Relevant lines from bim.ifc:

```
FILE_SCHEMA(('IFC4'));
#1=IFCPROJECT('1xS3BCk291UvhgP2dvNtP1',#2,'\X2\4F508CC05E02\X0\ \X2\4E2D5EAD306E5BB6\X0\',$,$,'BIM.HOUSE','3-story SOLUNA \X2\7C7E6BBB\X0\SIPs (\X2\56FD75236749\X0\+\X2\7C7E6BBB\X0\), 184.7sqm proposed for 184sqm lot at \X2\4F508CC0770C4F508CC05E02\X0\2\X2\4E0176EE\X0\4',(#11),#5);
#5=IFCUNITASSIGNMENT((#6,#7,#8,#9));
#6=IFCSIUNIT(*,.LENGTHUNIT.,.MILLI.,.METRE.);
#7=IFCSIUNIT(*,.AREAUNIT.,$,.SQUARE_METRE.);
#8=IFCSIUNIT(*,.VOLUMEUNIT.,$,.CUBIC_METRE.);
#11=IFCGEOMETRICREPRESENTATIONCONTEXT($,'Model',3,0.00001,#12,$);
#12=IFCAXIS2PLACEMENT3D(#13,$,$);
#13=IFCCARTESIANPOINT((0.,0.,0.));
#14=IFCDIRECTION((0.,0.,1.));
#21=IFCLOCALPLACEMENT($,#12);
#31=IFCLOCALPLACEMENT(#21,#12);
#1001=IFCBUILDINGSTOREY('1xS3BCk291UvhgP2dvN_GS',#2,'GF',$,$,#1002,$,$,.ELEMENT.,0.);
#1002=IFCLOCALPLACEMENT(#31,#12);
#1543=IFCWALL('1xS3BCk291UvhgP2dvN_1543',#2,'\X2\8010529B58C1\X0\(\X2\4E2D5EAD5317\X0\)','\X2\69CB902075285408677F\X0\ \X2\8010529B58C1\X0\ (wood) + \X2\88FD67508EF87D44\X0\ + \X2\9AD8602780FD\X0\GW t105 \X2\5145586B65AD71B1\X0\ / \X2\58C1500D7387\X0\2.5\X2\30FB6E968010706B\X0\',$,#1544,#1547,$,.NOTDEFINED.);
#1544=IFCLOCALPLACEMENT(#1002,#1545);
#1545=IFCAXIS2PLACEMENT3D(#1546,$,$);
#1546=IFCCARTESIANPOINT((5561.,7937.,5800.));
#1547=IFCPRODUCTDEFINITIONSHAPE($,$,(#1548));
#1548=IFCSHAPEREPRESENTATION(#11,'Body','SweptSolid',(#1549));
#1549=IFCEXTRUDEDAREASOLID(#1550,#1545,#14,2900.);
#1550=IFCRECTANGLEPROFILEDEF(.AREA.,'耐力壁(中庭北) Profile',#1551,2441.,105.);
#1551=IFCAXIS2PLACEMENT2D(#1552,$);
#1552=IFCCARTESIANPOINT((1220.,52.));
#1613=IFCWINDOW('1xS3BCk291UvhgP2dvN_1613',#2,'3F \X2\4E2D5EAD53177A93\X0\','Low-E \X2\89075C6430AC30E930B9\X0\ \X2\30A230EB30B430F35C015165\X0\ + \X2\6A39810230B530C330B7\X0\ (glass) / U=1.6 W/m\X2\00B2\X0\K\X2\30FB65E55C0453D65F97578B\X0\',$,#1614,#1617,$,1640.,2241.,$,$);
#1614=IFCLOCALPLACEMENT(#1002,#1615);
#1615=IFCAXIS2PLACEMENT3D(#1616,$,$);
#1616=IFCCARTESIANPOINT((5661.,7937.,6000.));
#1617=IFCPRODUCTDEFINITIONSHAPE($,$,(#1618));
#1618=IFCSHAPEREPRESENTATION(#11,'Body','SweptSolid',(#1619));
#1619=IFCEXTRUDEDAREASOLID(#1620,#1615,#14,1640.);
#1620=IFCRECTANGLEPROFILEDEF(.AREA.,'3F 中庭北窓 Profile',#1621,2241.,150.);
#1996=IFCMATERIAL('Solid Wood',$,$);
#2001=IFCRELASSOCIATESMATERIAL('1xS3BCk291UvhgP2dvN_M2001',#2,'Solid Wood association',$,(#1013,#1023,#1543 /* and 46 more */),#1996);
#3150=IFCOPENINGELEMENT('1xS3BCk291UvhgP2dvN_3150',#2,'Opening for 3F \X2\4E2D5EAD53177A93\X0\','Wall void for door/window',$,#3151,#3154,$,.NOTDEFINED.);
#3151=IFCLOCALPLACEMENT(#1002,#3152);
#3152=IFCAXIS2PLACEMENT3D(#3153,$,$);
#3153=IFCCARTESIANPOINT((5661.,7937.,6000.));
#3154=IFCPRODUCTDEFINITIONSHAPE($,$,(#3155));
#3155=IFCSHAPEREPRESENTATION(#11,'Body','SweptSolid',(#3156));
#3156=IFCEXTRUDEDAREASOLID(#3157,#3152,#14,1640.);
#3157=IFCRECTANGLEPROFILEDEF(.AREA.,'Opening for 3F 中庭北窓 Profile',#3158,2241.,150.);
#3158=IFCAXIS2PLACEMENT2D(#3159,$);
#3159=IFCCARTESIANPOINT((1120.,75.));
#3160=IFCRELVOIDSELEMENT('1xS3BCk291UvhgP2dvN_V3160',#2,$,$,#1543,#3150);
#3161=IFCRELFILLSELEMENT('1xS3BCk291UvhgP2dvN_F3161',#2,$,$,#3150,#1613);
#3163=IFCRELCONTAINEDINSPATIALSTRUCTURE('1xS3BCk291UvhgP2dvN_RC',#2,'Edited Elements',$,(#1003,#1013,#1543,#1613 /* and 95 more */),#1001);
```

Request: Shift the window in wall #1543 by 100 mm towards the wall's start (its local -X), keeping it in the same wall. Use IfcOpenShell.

```python
import ifcopenshell
import ifcopenshell.api.geometry
import ifcopenshell.util.placement
import ifcopenshell.util.unit

model = ifcopenshell.open("bim.ifc")
unit_scale = ifcopenshell.util.unit.calculate_unit_scale(model)

window = model.by_id(1613)
opening = window.FillsVoids[0].RelatingOpeningElement
wall = opening.VoidsElements[0].RelatingBuildingElement

wall_matrix = ifcopenshell.util.placement.get_local_placement(wall.ObjectPlacement)
shift = wall_matrix[:3, 0] * -0.1 / unit_scale
before = ifcopenshell.util.placement.get_local_placement(window.ObjectPlacement)[:3, 3].copy()

# The window is not placed relative to its opening, so move both.
for product in (opening, window):
    matrix = ifcopenshell.util.placement.get_local_placement(product.ObjectPlacement)
    matrix[:3, 3] += shift
    ifcopenshell.api.geometry.edit_object_placement(model, product=product, matrix=matrix, is_si=False)

after = ifcopenshell.util.placement.get_local_placement(window.ObjectPlacement)[:3, 3]
print("window moved by", (after - before).round(3) + 0.0)

model.write("bim_v2.ifc")
```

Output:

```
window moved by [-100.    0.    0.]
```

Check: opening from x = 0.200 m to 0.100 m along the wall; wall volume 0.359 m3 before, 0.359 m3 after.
